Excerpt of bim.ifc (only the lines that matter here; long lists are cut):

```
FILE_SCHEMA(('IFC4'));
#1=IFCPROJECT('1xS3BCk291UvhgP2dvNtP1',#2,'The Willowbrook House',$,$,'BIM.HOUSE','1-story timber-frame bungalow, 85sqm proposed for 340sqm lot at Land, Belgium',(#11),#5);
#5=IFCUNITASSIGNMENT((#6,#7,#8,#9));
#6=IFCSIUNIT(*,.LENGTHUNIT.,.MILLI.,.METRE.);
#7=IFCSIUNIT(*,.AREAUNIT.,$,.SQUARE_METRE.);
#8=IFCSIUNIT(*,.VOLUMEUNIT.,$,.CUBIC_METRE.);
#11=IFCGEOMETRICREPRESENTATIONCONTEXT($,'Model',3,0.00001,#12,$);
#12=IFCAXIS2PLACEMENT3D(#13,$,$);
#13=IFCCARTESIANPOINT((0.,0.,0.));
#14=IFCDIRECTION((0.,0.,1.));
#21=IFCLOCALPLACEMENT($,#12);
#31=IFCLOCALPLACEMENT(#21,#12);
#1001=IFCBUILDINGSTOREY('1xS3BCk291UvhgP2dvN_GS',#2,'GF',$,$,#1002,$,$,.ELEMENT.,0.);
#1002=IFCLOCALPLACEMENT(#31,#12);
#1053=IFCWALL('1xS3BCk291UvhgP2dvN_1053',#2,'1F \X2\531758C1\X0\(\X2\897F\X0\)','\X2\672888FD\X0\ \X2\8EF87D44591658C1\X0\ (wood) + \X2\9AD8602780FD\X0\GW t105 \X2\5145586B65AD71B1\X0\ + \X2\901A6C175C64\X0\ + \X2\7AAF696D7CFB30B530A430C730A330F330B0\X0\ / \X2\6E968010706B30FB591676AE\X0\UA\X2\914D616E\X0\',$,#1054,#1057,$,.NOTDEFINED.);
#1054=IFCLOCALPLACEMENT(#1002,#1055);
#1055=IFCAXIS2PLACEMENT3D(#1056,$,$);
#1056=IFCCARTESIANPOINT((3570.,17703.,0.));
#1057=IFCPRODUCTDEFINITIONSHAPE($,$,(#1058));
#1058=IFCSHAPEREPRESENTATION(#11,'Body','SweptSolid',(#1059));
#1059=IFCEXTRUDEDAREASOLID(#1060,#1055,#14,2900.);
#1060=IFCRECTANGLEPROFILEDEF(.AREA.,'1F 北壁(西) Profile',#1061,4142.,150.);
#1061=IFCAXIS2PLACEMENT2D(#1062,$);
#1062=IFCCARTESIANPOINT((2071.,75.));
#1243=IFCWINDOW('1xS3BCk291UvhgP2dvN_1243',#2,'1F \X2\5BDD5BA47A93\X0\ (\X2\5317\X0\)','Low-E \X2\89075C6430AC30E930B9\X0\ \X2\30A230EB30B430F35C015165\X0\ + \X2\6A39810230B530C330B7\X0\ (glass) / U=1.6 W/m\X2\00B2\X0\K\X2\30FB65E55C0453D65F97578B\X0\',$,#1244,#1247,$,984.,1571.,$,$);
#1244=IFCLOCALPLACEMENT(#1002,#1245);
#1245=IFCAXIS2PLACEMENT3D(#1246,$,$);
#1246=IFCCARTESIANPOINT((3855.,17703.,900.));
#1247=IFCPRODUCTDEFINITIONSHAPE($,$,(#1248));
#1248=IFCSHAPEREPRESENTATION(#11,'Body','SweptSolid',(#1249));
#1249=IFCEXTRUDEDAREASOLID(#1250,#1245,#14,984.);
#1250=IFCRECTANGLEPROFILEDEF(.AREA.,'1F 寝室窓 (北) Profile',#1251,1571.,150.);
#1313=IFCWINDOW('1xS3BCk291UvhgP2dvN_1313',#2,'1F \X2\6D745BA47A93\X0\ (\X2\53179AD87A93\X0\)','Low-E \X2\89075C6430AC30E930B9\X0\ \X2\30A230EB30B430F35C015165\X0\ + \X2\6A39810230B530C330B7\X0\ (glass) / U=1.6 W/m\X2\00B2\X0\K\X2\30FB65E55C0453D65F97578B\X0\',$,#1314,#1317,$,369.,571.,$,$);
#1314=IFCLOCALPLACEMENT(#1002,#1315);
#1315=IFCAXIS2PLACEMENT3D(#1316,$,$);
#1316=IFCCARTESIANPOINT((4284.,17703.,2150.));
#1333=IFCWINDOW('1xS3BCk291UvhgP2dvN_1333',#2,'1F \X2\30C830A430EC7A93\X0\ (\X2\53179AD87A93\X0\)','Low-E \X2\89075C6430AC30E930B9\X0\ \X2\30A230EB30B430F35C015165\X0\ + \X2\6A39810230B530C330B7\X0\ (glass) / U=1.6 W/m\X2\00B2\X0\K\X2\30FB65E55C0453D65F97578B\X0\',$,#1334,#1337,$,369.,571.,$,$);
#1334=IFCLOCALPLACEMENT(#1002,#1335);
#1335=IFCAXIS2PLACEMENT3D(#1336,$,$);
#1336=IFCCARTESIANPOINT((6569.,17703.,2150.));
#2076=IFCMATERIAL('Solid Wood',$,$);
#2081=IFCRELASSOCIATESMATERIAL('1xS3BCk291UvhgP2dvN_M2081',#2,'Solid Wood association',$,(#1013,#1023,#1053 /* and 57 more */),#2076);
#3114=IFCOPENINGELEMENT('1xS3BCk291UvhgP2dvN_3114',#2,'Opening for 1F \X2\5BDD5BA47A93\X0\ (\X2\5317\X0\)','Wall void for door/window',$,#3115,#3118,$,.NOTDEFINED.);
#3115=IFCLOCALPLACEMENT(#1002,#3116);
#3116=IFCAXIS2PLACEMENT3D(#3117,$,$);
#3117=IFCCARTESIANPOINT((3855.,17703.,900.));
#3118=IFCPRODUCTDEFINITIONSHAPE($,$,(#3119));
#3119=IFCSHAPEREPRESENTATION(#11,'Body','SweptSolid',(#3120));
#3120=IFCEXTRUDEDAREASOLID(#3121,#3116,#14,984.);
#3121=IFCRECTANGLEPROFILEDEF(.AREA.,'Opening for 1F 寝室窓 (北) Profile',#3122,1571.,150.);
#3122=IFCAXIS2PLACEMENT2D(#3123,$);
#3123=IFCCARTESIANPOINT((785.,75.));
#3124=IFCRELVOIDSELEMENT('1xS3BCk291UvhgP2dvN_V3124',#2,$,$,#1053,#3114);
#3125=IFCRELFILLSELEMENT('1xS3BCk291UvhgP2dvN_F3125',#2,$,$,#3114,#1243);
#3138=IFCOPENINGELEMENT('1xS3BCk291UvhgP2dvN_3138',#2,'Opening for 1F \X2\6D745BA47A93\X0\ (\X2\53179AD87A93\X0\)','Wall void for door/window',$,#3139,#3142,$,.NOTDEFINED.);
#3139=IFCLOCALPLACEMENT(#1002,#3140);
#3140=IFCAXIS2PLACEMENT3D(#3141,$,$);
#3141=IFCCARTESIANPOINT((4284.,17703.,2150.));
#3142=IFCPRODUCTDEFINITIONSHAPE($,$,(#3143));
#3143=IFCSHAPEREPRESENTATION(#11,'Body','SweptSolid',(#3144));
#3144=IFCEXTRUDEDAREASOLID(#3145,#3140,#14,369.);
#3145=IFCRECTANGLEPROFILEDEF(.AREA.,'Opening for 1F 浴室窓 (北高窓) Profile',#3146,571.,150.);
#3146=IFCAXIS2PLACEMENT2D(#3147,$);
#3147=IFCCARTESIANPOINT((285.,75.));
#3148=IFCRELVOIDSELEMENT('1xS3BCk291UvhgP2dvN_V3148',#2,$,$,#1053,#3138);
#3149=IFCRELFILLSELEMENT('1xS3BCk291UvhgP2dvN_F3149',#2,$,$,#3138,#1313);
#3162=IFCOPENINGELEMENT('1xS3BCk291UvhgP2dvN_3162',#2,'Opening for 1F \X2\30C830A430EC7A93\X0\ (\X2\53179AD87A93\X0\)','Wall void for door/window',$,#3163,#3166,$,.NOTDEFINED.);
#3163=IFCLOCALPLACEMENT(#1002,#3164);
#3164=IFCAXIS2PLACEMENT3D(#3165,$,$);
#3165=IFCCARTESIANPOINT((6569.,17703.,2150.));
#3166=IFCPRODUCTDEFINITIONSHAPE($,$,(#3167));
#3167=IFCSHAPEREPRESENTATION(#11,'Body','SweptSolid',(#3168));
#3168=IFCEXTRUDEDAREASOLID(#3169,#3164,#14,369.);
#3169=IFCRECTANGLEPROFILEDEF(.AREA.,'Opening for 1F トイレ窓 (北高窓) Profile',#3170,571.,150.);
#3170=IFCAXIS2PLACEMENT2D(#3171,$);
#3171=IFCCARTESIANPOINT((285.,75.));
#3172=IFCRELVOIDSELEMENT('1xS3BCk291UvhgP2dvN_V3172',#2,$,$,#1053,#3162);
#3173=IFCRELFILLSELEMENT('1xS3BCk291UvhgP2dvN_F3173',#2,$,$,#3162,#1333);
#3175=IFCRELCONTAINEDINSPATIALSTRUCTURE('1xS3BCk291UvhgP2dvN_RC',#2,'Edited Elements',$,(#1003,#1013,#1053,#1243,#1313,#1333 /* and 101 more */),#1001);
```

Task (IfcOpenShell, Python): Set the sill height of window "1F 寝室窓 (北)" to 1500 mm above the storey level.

```python
import numpy as np
import ifcopenshell
import ifcopenshell.api.geometry
import ifcopenshell.geom
import ifcopenshell.util.element
import ifcopenshell.util.placement
import ifcopenshell.util.shape
import ifcopenshell.util.unit

model = ifcopenshell.open("bim.ifc")
unit_scale = ifcopenshell.util.unit.calculate_unit_scale(model)

window = model.by_guid("1xS3BCk291UvhgP2dvN_1243")
opening = window.FillsVoids[0].RelatingOpeningElement
storey = ifcopenshell.util.element.get_container(window, ifc_class="IfcBuildingStorey")
level = ifcopenshell.util.placement.get_local_placement(storey.ObjectPlacement)[2, 3]

# The opening's origin need not be at the sill, so measure its lowest point.
shape = ifcopenshell.geom.create_shape(ifcopenshell.geom.settings(), opening)
bottom = ifcopenshell.util.shape.get_shape_bottom_elevation(shape, shape.geometry) / unit_scale
dz = level + 1.5 / unit_scale - bottom

shift = np.array([0.0, 0.0, dz])
# The window is not placed relative to its opening, so move both.
for product in (opening, window):
    matrix = ifcopenshell.util.placement.get_local_placement(product.ObjectPlacement)
    matrix[:3, 3] += shift
    ifcopenshell.api.geometry.edit_object_placement(model, product=product, matrix=matrix, is_si=False)

print(f"moved by {dz * unit_scale:+.3f} m")

model.write("bim-out.ifc")
```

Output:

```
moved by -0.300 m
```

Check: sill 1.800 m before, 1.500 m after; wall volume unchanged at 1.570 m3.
